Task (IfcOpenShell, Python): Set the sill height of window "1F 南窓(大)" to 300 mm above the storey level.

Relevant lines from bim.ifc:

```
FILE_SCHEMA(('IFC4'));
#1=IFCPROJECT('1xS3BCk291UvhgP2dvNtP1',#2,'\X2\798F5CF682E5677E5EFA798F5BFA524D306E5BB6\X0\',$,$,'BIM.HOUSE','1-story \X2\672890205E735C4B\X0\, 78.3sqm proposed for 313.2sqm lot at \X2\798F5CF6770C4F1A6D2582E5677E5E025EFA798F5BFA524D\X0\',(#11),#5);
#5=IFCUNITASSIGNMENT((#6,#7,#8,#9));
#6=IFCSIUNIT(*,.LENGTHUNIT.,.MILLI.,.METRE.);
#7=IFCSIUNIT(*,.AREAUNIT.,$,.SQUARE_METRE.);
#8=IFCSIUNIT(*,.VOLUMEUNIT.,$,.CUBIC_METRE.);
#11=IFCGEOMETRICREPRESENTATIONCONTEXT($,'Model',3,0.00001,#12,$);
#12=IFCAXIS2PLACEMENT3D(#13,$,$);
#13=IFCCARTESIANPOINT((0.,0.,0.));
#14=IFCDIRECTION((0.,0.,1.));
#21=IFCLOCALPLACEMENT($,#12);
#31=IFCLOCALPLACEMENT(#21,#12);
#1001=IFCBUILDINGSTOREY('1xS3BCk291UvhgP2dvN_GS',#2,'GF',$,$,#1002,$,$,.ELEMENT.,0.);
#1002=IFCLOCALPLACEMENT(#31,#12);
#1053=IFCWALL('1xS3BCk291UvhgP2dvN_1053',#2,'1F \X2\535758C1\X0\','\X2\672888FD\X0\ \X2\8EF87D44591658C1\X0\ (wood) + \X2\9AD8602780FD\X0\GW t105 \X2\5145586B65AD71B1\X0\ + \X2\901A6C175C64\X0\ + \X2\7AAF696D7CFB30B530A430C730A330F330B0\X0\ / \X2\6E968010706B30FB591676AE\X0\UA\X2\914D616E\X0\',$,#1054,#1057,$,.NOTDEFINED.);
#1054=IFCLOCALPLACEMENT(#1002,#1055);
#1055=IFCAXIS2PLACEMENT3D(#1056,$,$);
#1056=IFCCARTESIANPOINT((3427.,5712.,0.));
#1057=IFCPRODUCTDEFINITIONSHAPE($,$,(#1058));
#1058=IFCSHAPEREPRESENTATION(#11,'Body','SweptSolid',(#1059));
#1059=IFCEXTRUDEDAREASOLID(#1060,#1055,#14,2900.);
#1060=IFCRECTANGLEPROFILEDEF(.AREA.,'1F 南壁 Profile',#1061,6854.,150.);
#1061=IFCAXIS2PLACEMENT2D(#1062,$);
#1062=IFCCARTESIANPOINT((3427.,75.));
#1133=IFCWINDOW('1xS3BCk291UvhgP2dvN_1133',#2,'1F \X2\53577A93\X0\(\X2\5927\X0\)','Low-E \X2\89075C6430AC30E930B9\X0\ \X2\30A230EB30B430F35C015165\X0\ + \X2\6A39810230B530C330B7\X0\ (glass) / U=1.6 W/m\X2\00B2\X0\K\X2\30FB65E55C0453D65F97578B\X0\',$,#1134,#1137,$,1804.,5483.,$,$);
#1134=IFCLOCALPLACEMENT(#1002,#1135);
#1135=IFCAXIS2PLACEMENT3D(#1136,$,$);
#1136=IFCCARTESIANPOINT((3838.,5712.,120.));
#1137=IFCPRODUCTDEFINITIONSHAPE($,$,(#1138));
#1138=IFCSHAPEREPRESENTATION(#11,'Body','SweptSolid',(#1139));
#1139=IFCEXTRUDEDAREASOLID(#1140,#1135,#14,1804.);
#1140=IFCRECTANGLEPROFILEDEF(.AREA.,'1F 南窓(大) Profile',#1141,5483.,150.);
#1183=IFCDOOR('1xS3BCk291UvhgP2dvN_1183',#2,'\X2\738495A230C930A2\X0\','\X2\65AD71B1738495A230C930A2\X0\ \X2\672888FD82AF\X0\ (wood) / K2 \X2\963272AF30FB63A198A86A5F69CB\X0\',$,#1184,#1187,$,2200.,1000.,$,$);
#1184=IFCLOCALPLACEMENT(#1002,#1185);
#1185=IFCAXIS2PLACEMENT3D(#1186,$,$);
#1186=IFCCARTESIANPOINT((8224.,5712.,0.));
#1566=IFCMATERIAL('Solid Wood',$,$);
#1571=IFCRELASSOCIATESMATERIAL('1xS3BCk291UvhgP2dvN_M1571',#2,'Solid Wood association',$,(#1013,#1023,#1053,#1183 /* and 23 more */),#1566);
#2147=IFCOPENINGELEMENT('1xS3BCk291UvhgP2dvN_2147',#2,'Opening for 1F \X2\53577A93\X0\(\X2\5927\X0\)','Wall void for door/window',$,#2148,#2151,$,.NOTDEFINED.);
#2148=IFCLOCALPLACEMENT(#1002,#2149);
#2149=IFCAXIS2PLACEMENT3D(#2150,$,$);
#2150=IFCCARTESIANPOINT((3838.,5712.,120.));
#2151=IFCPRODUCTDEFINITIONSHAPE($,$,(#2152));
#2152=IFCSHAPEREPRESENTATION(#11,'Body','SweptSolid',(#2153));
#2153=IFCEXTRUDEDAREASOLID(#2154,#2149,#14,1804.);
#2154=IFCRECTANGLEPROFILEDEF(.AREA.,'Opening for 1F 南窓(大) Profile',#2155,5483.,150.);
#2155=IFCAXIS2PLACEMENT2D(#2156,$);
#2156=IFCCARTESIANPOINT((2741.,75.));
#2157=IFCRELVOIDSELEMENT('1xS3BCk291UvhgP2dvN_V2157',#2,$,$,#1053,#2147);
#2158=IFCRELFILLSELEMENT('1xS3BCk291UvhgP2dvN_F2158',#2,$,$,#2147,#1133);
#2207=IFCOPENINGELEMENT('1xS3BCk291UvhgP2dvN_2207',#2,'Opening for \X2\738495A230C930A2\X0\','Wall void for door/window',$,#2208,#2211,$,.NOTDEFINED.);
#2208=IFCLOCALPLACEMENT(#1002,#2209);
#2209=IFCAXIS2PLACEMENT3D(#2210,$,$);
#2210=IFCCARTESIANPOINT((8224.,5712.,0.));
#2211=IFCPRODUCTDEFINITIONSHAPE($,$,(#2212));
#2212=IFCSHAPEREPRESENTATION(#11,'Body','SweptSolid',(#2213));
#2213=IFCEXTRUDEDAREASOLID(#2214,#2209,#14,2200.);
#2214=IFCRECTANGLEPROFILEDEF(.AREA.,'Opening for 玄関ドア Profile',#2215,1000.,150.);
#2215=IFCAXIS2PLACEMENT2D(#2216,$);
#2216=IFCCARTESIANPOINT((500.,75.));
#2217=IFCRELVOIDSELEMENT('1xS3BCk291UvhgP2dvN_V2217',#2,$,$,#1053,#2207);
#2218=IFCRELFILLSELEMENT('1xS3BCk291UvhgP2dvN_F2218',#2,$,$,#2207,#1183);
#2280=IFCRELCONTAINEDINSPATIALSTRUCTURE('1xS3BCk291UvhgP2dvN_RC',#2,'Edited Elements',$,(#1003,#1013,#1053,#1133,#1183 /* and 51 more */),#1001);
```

```python
import numpy as np
import ifcopenshell
import ifcopenshell.api.geometry
import ifcopenshell.geom
import ifcopenshell.util.element
import ifcopenshell.util.placement
import ifcopenshell.util.shape
import ifcopenshell.util.unit

model = ifcopenshell.open("bim.ifc")
unit_scale = ifcopenshell.util.unit.calculate_unit_scale(model)

window = model.by_guid("1xS3BCk291UvhgP2dvN_1133")
opening = window.FillsVoids[0].RelatingOpeningElement
storey = ifcopenshell.util.element.get_container(window, ifc_class="IfcBuildingStorey")
level = ifcopenshell.util.placement.get_local_placement(storey.ObjectPlacement)[2, 3]

# The opening's origin need not be at the sill, so measure its lowest point.
shape = ifcopenshell.geom.create_shape(ifcopenshell.geom.settings(), opening)
bottom = ifcopenshell.util.shape.get_shape_bottom_elevation(shape, shape.geometry) / unit_scale
dz = level + 0.3 / unit_scale - bottom

shift = np.array([0.0, 0.0, dz])
# The window is not placed relative to its opening, so move both.
for product in (opening, window):
    matrix = ifcopenshell.util.placement.get_local_placement(product.ObjectPlacement)
    matrix[:3, 3] += shift
    ifcopenshell.api.geometry.edit_object_placement(model, product=product, matrix=matrix, is_si=False)

print(f"moved by {dz * unit_scale:+.3f} m")

model.write("bim_updated.ifc")
```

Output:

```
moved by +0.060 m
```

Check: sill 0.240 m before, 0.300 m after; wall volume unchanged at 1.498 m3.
